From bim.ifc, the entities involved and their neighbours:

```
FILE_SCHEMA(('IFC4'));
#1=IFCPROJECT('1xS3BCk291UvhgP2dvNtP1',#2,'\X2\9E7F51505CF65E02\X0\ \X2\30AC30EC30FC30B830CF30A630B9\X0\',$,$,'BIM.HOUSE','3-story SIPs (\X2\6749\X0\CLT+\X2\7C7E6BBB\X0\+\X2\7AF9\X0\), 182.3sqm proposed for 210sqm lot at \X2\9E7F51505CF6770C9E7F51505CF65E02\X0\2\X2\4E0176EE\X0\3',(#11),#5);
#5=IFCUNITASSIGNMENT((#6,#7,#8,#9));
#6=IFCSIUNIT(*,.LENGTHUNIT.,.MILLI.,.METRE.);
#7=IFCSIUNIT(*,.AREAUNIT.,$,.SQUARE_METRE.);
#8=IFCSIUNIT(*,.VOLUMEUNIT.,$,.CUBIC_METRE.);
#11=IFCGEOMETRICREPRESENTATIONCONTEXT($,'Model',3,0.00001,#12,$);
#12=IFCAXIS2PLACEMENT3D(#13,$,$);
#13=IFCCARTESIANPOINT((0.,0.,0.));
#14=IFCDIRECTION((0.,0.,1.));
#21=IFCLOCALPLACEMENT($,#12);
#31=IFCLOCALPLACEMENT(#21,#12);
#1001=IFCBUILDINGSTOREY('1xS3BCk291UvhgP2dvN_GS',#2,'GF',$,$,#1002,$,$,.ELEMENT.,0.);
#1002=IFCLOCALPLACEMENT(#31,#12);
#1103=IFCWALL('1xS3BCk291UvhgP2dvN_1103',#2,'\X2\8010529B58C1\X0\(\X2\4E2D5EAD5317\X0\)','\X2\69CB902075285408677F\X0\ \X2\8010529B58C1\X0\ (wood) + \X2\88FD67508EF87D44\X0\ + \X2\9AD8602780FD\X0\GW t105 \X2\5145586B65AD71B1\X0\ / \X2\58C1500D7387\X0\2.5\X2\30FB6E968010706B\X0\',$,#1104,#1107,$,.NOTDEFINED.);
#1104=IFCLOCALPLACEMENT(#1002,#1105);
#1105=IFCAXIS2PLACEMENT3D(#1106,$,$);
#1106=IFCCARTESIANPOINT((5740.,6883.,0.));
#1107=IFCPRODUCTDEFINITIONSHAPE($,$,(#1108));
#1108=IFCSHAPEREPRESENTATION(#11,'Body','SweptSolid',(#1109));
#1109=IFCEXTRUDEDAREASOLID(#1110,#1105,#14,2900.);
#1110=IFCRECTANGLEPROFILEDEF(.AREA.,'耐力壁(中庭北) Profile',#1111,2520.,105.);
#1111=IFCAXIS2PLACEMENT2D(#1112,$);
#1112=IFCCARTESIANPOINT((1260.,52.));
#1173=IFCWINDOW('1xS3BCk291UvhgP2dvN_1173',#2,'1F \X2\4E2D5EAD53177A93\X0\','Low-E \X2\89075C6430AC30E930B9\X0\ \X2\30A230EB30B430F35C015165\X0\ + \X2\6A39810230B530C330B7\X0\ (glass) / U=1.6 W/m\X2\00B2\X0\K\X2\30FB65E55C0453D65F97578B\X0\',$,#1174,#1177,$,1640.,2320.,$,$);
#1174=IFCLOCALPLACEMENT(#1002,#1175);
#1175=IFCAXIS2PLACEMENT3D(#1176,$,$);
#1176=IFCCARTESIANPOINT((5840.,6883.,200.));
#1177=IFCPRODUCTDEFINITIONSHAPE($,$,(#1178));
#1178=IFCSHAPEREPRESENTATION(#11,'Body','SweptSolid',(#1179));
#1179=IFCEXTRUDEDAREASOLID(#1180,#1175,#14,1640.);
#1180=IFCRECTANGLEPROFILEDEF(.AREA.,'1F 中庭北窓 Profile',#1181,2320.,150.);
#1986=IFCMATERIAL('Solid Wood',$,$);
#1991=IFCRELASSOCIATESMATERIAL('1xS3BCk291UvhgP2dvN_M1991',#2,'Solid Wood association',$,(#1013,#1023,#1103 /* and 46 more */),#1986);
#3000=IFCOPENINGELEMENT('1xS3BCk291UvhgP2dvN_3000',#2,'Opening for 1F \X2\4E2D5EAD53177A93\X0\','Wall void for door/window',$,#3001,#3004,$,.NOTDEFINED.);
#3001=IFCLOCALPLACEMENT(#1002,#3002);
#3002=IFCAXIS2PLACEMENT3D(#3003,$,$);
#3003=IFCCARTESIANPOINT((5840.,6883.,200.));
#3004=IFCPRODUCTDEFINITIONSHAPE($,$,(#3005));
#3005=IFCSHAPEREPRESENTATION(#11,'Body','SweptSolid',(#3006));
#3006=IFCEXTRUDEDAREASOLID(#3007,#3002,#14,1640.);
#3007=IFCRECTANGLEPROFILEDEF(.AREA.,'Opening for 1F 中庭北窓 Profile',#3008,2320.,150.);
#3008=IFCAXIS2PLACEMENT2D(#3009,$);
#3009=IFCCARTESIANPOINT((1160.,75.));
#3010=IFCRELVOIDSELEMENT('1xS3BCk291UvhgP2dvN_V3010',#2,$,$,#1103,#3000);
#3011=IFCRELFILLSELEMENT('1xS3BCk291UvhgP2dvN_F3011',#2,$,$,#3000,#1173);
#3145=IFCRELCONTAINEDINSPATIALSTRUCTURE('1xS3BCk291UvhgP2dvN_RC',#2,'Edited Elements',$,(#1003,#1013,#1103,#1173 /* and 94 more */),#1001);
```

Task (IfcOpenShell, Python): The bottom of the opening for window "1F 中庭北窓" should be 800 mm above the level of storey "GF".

```python
import numpy as np
import ifcopenshell
import ifcopenshell.api.geometry
import ifcopenshell.geom
import ifcopenshell.util.element
import ifcopenshell.util.placement
import ifcopenshell.util.shape
import ifcopenshell.util.unit

model = ifcopenshell.open("bim.ifc")
unit_scale = ifcopenshell.util.unit.calculate_unit_scale(model)

window = model.by_guid("1xS3BCk291UvhgP2dvN_1173")
opening = window.FillsVoids[0].RelatingOpeningElement
storey = ifcopenshell.util.element.get_container(window, ifc_class="IfcBuildingStorey")
level = ifcopenshell.util.placement.get_local_placement(storey.ObjectPlacement)[2, 3]

# The opening's origin need not be at the sill, so measure its lowest point.
shape = ifcopenshell.geom.create_shape(ifcopenshell.geom.settings(), opening)
bottom = ifcopenshell.util.shape.get_shape_bottom_elevation(shape, shape.geometry) / unit_scale
dz = level + 0.8 / unit_scale - bottom

shift = np.array([0.0, 0.0, dz])
# The window is not placed relative to its opening, so move both.
for product in (opening, window):
    matrix = ifcopenshell.util.placement.get_local_placement(product.ObjectPlacement)
    matrix[:3, 3] += shift
    ifcopenshell.api.geometry.edit_object_placement(model, product=product, matrix=matrix, is_si=False)

print(f"moved by {dz * unit_scale:+.3f} m")

model.write("bim_v2.ifc")
```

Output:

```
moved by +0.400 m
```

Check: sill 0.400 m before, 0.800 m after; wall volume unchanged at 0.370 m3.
